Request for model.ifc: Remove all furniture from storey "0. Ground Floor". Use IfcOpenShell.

First a look at what the model holds.

```python
import ifcopenshell
import ifcopenshell.util.element

model = ifcopenshell.open("model.ifc")
print(model.schema)
storey = next(s for s in model.by_type("IfcBuildingStorey") if s.Name == "0. Ground Floor")
furniture = [e for e in ifcopenshell.util.element.get_decomposition(storey) if e.is_a("IfcFurnishingElement")]
seen = {}
for e in furniture:
    element_type = ifcopenshell.util.element.get_type(e)
    name = element_type.Name if element_type not in (None, e) else None
    seen[name] = seen.get(name, 0) + 1
for name, count in sorted(seen.items(), key=str):
    print(count, "x", name)
```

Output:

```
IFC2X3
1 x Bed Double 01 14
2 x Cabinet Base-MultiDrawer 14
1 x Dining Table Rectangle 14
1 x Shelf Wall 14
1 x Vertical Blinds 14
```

```python
import ifcopenshell
import ifcopenshell.api.root
import ifcopenshell.util.element

model = ifcopenshell.open("model.ifc")

storey = next(s for s in model.by_type("IfcBuildingStorey") if s.Name == "0. Ground Floor")
furniture = [e for e in ifcopenshell.util.element.get_decomposition(storey) if e.is_a("IfcFurnishingElement")]

for e in furniture:
    ifcopenshell.api.root.remove_product(model, product=e)
print(len(furniture), "removed")

model.write("model_v2.ifc")
```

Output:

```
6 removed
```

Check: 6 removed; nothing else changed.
